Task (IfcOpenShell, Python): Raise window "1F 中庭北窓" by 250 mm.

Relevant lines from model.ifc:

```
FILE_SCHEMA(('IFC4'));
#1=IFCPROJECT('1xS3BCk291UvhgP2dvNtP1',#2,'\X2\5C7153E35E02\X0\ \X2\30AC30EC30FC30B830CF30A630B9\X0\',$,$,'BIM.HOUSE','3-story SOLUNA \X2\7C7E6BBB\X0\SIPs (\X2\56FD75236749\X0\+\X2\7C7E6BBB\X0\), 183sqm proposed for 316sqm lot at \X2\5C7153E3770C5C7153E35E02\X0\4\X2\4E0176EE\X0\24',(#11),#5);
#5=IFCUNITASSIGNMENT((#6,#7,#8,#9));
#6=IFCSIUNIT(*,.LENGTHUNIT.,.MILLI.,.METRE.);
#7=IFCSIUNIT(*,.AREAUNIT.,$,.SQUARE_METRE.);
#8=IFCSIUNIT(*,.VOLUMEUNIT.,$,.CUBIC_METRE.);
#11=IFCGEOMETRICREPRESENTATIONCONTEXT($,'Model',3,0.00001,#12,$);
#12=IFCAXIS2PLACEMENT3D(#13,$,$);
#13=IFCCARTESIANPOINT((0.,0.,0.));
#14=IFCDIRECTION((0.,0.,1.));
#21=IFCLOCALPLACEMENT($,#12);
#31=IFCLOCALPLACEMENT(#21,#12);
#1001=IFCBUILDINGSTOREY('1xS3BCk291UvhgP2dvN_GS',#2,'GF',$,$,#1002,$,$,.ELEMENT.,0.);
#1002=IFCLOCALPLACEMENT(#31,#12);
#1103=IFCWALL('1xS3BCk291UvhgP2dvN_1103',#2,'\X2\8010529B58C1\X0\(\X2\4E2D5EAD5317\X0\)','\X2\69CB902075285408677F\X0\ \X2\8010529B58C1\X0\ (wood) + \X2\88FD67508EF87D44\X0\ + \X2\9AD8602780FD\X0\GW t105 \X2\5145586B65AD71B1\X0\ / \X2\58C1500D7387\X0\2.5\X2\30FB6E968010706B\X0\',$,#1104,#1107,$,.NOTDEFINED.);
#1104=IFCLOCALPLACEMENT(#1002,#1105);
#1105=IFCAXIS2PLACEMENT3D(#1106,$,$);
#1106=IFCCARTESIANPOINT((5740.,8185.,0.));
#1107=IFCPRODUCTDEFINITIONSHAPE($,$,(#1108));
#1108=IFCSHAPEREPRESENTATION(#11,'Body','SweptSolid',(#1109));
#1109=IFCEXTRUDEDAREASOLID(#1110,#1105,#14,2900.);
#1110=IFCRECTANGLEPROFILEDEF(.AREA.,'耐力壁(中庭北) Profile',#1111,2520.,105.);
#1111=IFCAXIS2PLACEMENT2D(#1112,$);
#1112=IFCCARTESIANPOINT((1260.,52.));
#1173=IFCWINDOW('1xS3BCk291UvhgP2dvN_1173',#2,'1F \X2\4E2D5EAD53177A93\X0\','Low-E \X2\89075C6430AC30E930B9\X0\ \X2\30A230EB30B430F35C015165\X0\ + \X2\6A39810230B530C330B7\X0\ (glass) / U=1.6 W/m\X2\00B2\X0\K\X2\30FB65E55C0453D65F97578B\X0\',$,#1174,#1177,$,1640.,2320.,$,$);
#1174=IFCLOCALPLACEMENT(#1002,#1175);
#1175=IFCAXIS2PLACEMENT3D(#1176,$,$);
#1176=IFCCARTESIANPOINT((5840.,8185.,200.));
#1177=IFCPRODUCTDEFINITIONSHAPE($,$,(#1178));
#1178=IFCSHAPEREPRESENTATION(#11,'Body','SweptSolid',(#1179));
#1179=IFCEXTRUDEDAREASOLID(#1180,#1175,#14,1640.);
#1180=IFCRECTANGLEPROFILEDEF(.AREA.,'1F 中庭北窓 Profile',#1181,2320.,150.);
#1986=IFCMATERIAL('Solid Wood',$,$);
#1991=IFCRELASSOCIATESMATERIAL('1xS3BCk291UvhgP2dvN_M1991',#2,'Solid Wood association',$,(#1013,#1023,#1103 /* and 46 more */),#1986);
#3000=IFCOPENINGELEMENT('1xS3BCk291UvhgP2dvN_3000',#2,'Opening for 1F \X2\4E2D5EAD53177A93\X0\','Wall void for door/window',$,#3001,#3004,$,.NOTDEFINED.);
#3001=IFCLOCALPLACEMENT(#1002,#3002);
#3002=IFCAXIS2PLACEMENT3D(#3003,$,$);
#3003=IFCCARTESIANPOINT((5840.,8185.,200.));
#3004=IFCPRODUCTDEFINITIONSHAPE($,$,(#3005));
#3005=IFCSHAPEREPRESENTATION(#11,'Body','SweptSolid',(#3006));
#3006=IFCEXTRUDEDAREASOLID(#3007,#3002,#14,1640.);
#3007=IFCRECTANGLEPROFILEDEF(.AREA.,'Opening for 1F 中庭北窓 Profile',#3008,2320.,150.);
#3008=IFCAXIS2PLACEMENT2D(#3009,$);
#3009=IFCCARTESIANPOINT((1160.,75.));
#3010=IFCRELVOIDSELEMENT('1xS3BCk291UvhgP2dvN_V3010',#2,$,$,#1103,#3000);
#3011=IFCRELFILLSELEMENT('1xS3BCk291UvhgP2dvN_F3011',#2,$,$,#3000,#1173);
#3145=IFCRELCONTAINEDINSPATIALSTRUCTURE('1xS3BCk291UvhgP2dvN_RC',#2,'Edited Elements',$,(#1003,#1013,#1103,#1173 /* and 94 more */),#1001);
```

```python
import numpy as np
import ifcopenshell
import ifcopenshell.api.geometry
import ifcopenshell.util.placement
import ifcopenshell.util.unit

model = ifcopenshell.open("model.ifc")
unit_scale = ifcopenshell.util.unit.calculate_unit_scale(model)

window = model.by_guid("1xS3BCk291UvhgP2dvN_1173")
opening = window.FillsVoids[0].RelatingOpeningElement
dz = 0.25 / unit_scale

shift = np.array([0.0, 0.0, dz])
# The window is not placed relative to its opening, so move both.
for product in (opening, window):
    matrix = ifcopenshell.util.placement.get_local_placement(product.ObjectPlacement)
    matrix[:3, 3] += shift
    ifcopenshell.api.geometry.edit_object_placement(model, product=product, matrix=matrix, is_si=False)

print(f"moved by {dz * unit_scale:+.3f} m")

model.write("model_edited.ifc")
```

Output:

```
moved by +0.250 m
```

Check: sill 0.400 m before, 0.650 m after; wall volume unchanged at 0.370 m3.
